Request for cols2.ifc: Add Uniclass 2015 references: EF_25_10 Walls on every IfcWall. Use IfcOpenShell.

First a look at what the model holds.

```python
import ifcopenshell

model = ifcopenshell.open("cols2.ifc")
print(model.schema)
print("classifications:", [c.Name for c in model.by_type("IfcClassification")])
for ifc_class in ("IfcDoor", "IfcRoof", "IfcStair", "IfcWall", "IfcWindow"):
    print(ifc_class, len(model.by_type(ifc_class)))
```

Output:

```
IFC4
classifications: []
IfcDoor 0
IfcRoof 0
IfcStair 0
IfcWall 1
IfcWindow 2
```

```python
import ifcopenshell
import ifcopenshell.api.classification

model = ifcopenshell.open("cols2.ifc")

system = ifcopenshell.api.classification.add_classification(model, classification="Uniclass 2015")

codes = {
    "IfcWall": ("EF_25_10", "Walls"),
}
for ifc_class, (code, name) in codes.items():
    products = model.by_type(ifc_class)
    ifcopenshell.api.classification.add_reference(
        model, products=products, classification=system, identification=code, name=name
    )
    print(code, len(products))

model.write("cols2-out.ifc")
```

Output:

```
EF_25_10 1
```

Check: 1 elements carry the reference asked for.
